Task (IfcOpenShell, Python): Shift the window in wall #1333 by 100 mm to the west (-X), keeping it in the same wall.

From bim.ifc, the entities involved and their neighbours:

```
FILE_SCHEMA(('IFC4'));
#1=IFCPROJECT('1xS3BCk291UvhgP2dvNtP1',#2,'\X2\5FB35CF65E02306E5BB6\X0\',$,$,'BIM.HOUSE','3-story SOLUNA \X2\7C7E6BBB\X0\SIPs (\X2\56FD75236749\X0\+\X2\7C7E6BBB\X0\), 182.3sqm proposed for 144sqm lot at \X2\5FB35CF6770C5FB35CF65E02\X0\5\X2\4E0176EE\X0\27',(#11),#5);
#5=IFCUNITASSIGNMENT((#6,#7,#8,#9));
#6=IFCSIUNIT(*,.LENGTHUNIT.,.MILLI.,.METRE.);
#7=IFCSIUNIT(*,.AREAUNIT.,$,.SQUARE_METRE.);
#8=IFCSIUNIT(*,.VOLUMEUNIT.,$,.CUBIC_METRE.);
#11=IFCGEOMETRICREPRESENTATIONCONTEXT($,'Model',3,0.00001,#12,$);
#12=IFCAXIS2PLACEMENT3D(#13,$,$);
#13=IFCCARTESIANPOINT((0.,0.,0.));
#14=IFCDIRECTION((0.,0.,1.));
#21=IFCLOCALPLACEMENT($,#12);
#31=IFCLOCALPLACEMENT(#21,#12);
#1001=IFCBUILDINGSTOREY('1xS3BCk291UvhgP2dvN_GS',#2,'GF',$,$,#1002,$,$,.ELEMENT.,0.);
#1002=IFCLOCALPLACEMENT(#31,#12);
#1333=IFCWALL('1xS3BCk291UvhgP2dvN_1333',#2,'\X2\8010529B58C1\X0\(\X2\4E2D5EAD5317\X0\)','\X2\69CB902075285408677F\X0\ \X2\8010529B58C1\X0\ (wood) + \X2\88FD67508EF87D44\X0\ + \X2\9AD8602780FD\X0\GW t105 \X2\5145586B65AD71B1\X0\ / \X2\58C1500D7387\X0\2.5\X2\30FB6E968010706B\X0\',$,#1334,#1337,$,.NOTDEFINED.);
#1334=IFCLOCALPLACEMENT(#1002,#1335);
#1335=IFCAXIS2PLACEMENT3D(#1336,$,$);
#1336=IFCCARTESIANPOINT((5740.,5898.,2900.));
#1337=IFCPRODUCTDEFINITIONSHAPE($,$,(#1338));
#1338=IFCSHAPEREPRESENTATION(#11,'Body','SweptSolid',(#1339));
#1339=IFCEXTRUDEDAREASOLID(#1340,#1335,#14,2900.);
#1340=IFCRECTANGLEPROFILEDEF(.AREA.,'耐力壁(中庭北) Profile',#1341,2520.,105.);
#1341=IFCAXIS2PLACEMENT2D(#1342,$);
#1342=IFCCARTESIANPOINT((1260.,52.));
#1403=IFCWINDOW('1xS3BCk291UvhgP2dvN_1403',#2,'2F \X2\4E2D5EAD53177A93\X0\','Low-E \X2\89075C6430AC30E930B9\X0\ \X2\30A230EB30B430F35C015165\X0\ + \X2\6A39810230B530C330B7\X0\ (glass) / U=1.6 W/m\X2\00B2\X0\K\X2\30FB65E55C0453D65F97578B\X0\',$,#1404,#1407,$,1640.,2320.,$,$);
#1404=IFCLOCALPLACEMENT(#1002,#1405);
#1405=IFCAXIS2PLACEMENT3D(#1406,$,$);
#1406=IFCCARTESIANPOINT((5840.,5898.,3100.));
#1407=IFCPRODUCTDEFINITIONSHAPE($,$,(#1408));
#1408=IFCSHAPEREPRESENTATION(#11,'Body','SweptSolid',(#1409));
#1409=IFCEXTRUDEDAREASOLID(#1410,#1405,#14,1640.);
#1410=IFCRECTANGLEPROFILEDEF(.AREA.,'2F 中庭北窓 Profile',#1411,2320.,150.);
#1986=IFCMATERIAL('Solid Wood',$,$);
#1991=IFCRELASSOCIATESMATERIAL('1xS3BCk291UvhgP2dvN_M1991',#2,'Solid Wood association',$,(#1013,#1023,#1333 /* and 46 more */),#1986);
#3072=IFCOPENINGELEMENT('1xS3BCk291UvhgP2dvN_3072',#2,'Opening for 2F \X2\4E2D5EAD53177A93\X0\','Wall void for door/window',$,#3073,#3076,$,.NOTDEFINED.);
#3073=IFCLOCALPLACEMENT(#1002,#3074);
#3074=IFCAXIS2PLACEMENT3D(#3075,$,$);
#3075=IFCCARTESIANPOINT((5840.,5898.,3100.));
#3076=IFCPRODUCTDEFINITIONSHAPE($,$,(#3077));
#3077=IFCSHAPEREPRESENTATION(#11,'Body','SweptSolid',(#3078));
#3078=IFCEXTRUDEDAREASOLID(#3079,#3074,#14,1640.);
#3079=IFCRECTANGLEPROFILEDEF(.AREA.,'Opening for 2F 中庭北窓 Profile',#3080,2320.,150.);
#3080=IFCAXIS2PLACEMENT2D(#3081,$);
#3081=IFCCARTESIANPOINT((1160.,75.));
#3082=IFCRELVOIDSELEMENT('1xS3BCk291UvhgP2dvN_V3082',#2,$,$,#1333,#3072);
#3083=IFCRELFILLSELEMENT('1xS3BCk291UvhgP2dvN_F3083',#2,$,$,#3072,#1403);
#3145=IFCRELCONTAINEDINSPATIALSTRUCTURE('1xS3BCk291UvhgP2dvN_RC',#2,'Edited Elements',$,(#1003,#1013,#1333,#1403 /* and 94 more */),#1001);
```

```python
import ifcopenshell
import ifcopenshell.api.geometry
import ifcopenshell.util.placement

model = ifcopenshell.open("bim.ifc")

window = model.by_guid("1xS3BCk291UvhgP2dvN_1403")
opening = window.FillsVoids[0].RelatingOpeningElement
wall = opening.VoidsElements[0].RelatingBuildingElement

wall_matrix = ifcopenshell.util.placement.get_local_placement(wall.ObjectPlacement)
shift = wall_matrix[:3, 0] * -100.0
before = ifcopenshell.util.placement.get_local_placement(window.ObjectPlacement)[:3, 3].copy()

# The window is not placed relative to its opening, so move both.
for product in (opening, window):
    matrix = ifcopenshell.util.placement.get_local_placement(product.ObjectPlacement)
    matrix[:3, 3] += shift
    ifcopenshell.api.geometry.edit_object_placement(model, product=product, matrix=matrix, is_si=False)

after = ifcopenshell.util.placement.get_local_placement(window.ObjectPlacement)[:3, 3]
print("window moved by", (after - before).round(3) + 0.0)

model.write("bim_edited.ifc")
```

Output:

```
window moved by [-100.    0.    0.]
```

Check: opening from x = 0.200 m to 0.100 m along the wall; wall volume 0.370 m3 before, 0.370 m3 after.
